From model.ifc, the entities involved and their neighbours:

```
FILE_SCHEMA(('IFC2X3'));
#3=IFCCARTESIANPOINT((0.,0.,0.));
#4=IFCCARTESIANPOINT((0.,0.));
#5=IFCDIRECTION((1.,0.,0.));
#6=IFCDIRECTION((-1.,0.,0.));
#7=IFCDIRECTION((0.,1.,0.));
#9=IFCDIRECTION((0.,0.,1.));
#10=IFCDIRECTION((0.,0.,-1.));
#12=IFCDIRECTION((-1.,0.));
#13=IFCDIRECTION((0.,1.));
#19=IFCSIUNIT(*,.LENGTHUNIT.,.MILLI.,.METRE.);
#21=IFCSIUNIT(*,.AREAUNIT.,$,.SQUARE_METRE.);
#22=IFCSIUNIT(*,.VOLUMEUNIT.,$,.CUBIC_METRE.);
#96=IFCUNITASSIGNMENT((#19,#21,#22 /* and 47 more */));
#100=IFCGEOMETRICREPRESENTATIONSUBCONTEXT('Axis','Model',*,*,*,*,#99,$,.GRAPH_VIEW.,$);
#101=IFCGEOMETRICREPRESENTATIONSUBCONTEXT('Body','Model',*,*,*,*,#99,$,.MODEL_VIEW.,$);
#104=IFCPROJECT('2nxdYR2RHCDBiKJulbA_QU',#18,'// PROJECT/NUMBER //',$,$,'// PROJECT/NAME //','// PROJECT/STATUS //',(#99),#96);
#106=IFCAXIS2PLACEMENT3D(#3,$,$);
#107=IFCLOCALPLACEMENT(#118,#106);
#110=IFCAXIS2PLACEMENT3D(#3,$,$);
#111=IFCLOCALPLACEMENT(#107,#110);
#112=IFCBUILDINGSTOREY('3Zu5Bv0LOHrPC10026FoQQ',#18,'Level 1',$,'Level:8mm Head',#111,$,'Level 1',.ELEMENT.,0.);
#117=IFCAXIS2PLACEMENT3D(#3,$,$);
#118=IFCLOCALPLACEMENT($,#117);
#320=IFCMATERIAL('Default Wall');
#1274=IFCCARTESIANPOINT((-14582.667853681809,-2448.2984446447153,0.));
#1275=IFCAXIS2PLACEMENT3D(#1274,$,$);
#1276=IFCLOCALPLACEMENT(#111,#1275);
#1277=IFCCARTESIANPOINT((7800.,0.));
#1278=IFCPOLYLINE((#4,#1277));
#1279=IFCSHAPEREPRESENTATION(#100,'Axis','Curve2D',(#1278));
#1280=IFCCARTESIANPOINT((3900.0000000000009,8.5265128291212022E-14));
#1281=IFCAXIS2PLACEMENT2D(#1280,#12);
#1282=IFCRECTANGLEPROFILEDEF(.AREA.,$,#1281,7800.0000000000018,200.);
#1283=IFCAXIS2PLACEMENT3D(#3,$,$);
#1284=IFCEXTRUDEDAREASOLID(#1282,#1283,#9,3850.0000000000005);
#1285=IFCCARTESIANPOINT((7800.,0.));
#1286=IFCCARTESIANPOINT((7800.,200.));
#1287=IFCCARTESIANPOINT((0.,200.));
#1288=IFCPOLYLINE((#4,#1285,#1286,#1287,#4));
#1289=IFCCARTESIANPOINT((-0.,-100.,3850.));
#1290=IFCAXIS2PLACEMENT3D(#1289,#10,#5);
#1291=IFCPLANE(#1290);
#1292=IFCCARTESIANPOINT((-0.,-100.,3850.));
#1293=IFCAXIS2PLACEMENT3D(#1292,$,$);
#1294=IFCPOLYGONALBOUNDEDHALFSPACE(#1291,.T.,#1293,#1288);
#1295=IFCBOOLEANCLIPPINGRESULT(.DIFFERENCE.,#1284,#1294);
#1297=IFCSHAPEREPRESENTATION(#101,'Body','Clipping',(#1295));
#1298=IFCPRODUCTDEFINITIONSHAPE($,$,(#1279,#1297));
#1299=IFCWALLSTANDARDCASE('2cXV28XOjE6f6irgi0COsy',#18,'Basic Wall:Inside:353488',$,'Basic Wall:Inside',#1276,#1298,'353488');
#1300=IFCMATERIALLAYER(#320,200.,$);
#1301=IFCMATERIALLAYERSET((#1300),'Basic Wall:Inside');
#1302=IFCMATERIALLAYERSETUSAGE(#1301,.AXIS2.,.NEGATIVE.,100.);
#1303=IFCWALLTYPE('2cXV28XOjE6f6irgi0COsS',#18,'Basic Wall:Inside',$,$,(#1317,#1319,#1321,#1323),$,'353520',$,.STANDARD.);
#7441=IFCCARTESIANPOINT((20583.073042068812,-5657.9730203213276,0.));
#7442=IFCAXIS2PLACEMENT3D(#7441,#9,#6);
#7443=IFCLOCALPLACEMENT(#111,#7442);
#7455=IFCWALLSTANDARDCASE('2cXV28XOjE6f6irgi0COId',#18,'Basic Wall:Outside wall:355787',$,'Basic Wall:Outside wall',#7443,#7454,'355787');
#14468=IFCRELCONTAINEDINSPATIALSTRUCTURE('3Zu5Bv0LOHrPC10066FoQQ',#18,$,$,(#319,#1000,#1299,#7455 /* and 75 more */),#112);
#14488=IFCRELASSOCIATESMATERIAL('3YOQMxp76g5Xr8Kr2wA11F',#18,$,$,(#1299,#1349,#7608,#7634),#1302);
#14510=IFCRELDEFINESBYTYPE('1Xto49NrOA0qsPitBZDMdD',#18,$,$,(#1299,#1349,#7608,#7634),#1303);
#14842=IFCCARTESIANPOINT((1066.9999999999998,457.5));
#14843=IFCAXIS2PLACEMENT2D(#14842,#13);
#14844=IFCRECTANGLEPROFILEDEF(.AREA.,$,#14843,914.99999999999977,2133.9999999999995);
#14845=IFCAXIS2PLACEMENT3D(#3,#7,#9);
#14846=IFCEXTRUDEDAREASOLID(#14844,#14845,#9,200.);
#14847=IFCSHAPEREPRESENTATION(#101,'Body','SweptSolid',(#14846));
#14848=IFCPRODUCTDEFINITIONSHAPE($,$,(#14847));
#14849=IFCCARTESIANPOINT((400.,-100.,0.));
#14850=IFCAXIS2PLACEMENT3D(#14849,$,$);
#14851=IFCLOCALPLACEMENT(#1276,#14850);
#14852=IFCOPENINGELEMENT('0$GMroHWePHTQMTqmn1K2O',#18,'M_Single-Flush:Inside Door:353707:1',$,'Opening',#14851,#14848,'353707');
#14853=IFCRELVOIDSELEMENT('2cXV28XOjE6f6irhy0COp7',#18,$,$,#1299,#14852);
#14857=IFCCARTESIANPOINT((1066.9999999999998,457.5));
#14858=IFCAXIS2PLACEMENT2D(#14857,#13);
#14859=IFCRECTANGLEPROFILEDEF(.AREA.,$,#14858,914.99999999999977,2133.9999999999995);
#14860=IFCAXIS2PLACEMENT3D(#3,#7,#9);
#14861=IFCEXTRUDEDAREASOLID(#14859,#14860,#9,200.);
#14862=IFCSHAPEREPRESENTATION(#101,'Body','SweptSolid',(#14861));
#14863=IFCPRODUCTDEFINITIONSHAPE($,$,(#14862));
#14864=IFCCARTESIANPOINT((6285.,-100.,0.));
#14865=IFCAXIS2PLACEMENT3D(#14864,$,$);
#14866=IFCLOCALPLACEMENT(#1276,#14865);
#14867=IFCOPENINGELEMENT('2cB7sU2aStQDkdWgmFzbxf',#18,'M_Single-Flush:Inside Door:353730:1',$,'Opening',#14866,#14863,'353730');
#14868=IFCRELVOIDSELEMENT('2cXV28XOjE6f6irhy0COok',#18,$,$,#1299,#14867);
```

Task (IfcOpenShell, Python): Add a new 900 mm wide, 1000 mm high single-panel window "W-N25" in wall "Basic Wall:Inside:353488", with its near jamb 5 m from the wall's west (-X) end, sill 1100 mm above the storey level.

```python
import numpy as np
import ifcopenshell
import ifcopenshell.api.feature
import ifcopenshell.api.geometry
import ifcopenshell.api.root
import ifcopenshell.api.spatial
import ifcopenshell.api.type
import ifcopenshell.geom
import ifcopenshell.util.element
import ifcopenshell.util.placement
import ifcopenshell.util.representation
import ifcopenshell.util.shape
import ifcopenshell.util.unit

model = ifcopenshell.open("model.ifc")
unit_scale = ifcopenshell.util.unit.calculate_unit_scale(model)
settings = ifcopenshell.geom.settings()


def volume(element):
    """Net volume in cubic metres, openings subtracted."""
    shape = ifcopenshell.geom.create_shape(settings, element)
    return ifcopenshell.util.shape.get_volume(shape.geometry)


wall = model.by_guid("2cXV28XOjE6f6irgi0COsy")
storey = ifcopenshell.util.element.get_container(wall, ifc_class="IfcBuildingStorey")
context = ifcopenshell.util.representation.get_context(model, "Model", "Body", "MODEL_VIEW")
before = volume(wall)

width, height, from_end, sill = 0.9, 1, 5, 1.1  # metres

# The wall runs along its own X axis, and the end named is its -X end.
wall_shape = ifcopenshell.geom.create_shape(settings, wall)
x, y, z = ifcopenshell.util.shape.get_vertices(wall_shape.geometry).T
start = x.min() + from_end
face, thickness = float(y.min()), float(y.max() - y.min())
wall_matrix = ifcopenshell.util.placement.get_local_placement(wall.ObjectPlacement)
level = ifcopenshell.util.placement.get_local_placement(storey.ObjectPlacement)[2, 3]


def in_wall(x, y):
    """Placement at x, y metres in the wall's axes, at sill height."""
    matrix = wall_matrix.copy()
    matrix[:, 3] = wall_matrix @ np.array([x / unit_scale, y / unit_scale, 0.0, 1.0])
    matrix[2, 3] = level + sill / unit_scale
    return matrix


# Opening: a box that overshoots both wall faces by 50 mm.
opening = ifcopenshell.api.root.create_entity(model, ifc_class="IfcOpeningElement")
box = ifcopenshell.api.geometry.add_wall_representation(
    model, context=context, length=width, height=height, thickness=thickness + 0.1
)
ifcopenshell.api.geometry.assign_representation(model, product=opening, representation=box)
ifcopenshell.api.geometry.edit_object_placement(model, product=opening, matrix=in_wall(start, face - 0.05), is_si=False)
ifcopenshell.api.feature.add_feature(model, feature=opening, element=wall)

window = ifcopenshell.api.root.create_entity(model, ifc_class="IfcWindow", name="W-N25")
window.OverallWidth, window.OverallHeight = width / unit_scale, height / unit_scale
body = ifcopenshell.api.geometry.add_window_representation(
    model,
    context=context,
    overall_width=window.OverallWidth,
    overall_height=window.OverallHeight,
    partition_type="SINGLE_PANEL",
)
ifcopenshell.api.geometry.assign_representation(model, product=window, representation=body)
ifcopenshell.api.spatial.assign_container(model, products=[window], relating_structure=storey)
fills = ifcopenshell.api.feature.add_filling(model, opening=opening, element=window)
fills.OwnerHistory = window.OwnerHistory  # required in IFC2X3

# IFC2X3 keeps the operation on the window style.
style = ifcopenshell.api.root.create_entity(model, ifc_class="IfcWindowStyle", name="W-N25")
style.OperationType, style.ConstructionType = "SINGLE_PANEL", "NOTDEFINED"
style.ParameterTakesPrecedence = style.Sizeable = False
ifcopenshell.api.type.assign_type(model, related_objects=[window], relating_type=style)

# Centre the window in the wall's thickness.
ifcopenshell.api.geometry.edit_object_placement(model, product=window, matrix=in_wall(start, face), is_si=False)
window_shape = ifcopenshell.geom.create_shape(settings, window)
depth = ifcopenshell.util.shape.get_vertices(window_shape.geometry)[:, 1]
offset = face + thickness / 2 - (depth.min() + depth.max()) / 2
ifcopenshell.api.geometry.edit_object_placement(model, product=window, matrix=in_wall(start, offset), is_si=False)

after = volume(wall)

print(f"wall volume {before:.3f} -> {after:.3f} m3")

model.write("model_rev.ifc")
```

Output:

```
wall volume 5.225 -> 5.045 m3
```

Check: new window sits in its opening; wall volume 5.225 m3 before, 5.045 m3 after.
